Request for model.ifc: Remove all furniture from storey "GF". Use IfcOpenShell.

First a look at what the model holds.

```python
import ifcopenshell
import ifcopenshell.util.element

model = ifcopenshell.open("model.ifc")
print(model.schema)
storey = next(s for s in model.by_type("IfcBuildingStorey") if s.Name == "GF")
furniture = [e for e in ifcopenshell.util.element.get_decomposition(storey) if e.is_a("IfcFurnishingElement")]
seen = {}
for e in furniture:
    element_type = ifcopenshell.util.element.get_type(e)
    name = element_type.Name if element_type not in (None, e) else None
    seen[name] = seen.get(name, 0) + 1
for name, count in sorted(seen.items(), key=str):
    print(count, "x", name)
```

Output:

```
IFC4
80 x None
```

```python
import ifcopenshell
import ifcopenshell.api.root
import ifcopenshell.util.element

model = ifcopenshell.open("model.ifc")

storey = next(s for s in model.by_type("IfcBuildingStorey") if s.Name == "GF")
furniture = [e for e in ifcopenshell.util.element.get_decomposition(storey) if e.is_a("IfcFurnishingElement")]

for e in furniture:
    ifcopenshell.api.root.remove_product(model, product=e)
print(len(furniture), "removed")

model.write("model-out.ifc")
```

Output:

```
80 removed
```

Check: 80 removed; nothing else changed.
